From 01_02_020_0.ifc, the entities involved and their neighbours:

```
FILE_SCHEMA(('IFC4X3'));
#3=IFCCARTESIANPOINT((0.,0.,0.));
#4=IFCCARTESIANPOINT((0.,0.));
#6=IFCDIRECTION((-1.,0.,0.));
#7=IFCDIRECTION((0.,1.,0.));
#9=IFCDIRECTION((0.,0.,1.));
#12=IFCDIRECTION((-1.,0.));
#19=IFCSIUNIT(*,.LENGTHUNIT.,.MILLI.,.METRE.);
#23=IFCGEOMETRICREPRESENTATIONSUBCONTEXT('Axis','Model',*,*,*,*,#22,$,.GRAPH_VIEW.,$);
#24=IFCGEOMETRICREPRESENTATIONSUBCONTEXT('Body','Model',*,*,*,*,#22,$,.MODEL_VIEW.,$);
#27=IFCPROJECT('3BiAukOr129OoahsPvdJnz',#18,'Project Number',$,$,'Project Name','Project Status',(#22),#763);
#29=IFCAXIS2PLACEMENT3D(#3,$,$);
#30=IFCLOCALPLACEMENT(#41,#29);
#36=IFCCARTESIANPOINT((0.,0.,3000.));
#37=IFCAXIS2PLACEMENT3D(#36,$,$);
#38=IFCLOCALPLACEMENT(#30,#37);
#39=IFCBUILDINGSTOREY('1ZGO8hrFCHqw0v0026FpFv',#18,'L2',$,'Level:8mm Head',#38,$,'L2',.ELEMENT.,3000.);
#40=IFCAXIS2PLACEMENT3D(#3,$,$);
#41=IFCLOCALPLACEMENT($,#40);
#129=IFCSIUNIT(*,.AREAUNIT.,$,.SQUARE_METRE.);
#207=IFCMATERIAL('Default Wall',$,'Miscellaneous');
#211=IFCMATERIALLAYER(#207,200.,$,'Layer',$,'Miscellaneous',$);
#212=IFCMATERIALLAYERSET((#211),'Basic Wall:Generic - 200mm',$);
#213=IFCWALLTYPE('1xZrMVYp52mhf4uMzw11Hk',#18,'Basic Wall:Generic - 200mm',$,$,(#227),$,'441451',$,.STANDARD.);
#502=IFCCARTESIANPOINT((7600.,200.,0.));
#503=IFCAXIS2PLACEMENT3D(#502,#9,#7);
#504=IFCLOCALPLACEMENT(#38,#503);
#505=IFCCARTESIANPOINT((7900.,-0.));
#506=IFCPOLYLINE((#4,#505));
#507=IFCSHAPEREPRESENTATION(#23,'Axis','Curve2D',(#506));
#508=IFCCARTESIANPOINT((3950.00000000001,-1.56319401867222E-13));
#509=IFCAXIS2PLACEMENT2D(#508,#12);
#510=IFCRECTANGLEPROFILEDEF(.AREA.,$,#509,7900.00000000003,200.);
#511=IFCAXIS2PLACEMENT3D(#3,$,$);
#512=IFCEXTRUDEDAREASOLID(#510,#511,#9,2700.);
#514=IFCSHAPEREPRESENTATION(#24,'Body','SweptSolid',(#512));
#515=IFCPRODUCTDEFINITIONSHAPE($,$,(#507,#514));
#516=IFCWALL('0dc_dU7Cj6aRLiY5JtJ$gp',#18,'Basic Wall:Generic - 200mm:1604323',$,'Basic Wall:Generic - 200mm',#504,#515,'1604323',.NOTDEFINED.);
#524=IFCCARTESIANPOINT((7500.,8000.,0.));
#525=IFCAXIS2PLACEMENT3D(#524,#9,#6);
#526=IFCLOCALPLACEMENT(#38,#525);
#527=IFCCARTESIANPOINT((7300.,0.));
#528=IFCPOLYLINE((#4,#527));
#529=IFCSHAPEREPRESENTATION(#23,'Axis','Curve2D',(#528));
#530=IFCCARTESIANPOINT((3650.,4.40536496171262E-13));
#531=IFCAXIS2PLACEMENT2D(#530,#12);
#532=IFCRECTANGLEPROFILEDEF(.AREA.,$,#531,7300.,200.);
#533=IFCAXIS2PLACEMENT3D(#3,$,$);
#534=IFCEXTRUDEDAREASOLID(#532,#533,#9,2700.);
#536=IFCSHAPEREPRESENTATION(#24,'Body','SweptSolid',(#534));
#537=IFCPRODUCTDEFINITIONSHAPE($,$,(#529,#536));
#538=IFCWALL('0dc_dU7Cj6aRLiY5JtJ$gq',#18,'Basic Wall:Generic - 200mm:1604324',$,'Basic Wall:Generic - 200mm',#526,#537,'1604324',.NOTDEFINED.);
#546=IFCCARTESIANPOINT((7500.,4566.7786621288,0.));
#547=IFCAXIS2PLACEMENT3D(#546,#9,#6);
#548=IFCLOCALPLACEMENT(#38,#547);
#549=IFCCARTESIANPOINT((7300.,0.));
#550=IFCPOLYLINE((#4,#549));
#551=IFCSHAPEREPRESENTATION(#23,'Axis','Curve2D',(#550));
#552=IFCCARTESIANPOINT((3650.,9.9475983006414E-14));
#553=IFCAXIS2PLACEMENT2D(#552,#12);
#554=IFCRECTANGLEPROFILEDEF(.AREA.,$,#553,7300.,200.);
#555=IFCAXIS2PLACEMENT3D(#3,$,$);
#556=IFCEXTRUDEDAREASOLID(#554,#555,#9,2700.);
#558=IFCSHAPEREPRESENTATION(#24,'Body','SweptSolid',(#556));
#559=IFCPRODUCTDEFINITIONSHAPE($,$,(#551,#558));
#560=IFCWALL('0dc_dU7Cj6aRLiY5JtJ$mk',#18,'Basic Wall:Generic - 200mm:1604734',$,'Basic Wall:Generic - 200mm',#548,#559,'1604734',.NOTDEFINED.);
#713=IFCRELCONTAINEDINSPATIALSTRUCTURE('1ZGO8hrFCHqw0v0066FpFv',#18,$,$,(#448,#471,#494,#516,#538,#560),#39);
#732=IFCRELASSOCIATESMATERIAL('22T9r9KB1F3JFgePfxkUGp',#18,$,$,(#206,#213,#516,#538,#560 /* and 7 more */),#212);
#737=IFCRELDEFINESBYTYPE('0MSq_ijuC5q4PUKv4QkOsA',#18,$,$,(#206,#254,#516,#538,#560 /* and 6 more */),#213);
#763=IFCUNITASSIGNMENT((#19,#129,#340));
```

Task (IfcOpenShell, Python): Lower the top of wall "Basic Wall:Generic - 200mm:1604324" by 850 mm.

```python
import ifcopenshell
import ifcopenshell.geom
import ifcopenshell.util.representation
import ifcopenshell.util.shape
import ifcopenshell.util.unit

model = ifcopenshell.open("01_02_020_0.ifc")
unit_scale = ifcopenshell.util.unit.calculate_unit_scale(model)
settings = ifcopenshell.geom.settings()


def volume(element):
    """Net volume in cubic metres, openings subtracted."""
    shape = ifcopenshell.geom.create_shape(settings, element)
    return ifcopenshell.util.shape.get_volume(shape.geometry)


wall = model.by_guid("0dc_dU7Cj6aRLiY5JtJ$gq")
before = volume(wall)

body = ifcopenshell.util.representation.get_representation(wall, "Model", "Body")
solid = body.Items[0]
old_height = solid.Depth
solid.Depth -= 0.85 / unit_scale
after = volume(wall)

print(f"height {old_height:g} -> {solid.Depth:g}, volume {before:.3f} -> {after:.3f} m3")

model.write("01_02_020_0_v2.ifc")
```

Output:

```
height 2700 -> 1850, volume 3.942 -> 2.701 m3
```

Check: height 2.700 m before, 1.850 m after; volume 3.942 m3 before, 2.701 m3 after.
